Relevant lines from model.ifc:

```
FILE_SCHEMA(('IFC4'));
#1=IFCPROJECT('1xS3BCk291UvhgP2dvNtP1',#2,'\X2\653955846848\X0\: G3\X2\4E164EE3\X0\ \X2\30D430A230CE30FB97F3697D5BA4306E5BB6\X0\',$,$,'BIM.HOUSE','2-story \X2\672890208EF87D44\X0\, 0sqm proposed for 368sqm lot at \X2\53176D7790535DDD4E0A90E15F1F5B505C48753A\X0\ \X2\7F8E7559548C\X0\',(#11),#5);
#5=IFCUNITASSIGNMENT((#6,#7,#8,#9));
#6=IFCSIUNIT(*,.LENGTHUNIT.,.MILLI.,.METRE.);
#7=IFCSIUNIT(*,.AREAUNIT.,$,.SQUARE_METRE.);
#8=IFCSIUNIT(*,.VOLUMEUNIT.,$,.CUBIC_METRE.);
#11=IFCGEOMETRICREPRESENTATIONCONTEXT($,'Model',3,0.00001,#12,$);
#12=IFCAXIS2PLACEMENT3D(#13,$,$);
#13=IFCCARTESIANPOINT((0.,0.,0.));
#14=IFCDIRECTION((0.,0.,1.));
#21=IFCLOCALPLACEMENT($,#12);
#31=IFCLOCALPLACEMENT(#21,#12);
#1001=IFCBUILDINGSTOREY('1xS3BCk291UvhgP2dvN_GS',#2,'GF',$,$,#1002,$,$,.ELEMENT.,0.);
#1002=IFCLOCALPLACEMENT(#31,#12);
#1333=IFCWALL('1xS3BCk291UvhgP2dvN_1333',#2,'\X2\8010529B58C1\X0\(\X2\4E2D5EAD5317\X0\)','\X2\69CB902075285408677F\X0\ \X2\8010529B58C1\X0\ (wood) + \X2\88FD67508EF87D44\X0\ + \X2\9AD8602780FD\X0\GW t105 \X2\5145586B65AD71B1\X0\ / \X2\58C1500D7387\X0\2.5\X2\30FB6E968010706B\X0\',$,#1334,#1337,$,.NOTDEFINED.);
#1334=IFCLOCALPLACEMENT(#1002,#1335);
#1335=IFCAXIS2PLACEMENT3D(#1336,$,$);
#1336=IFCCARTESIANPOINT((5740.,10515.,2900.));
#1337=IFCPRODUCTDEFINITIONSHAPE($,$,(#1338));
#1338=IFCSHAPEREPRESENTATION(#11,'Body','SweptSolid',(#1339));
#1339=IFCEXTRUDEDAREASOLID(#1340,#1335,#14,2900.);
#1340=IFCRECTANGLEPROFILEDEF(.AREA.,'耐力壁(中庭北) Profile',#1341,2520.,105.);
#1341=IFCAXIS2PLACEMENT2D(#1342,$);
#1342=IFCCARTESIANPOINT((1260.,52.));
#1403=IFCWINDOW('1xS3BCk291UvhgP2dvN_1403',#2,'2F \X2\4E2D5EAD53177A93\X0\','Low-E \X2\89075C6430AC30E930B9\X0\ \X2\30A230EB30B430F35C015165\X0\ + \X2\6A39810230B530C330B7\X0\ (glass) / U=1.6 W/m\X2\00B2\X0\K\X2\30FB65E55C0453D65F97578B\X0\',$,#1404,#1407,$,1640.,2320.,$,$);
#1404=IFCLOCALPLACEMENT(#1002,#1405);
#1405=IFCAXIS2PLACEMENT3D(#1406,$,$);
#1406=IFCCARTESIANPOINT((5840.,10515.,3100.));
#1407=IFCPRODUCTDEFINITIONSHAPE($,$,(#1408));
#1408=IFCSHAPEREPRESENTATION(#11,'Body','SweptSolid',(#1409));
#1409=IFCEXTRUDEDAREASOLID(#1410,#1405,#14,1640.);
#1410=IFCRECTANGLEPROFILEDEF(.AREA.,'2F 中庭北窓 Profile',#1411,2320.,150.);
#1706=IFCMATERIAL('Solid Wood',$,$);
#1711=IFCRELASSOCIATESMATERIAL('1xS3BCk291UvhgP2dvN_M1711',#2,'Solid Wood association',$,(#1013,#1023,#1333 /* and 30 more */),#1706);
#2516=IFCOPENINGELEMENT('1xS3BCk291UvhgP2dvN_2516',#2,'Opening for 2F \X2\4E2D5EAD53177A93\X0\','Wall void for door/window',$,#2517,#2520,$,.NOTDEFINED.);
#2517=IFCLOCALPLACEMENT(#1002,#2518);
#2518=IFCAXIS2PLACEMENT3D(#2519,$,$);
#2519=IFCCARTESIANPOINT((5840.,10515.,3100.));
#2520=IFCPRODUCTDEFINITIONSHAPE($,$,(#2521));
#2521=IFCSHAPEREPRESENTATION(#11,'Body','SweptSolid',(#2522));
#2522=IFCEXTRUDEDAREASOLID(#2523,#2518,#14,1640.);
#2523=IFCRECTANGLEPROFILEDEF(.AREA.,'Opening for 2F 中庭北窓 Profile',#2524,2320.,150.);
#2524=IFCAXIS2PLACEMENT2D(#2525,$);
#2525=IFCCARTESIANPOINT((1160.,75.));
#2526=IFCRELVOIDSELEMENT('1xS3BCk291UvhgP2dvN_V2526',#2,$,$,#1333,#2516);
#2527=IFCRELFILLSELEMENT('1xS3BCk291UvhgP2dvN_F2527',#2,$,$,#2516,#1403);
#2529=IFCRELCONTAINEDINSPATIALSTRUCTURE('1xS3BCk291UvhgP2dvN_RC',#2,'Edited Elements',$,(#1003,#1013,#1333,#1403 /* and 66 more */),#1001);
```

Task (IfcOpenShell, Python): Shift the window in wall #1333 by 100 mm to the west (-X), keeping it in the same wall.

```python
import ifcopenshell
import ifcopenshell.api.geometry
import ifcopenshell.util.placement
import ifcopenshell.util.unit

model = ifcopenshell.open("model.ifc")
unit_scale = ifcopenshell.util.unit.calculate_unit_scale(model)

window = model.by_id(1403)
opening = window.FillsVoids[0].RelatingOpeningElement
wall = opening.VoidsElements[0].RelatingBuildingElement

wall_matrix = ifcopenshell.util.placement.get_local_placement(wall.ObjectPlacement)
shift = wall_matrix[:3, 0] * -0.1 / unit_scale
before = ifcopenshell.util.placement.get_local_placement(window.ObjectPlacement)[:3, 3].copy()

# The window is not placed relative to its opening, so move both.
for product in (opening, window):
    matrix = ifcopenshell.util.placement.get_local_placement(product.ObjectPlacement)
    matrix[:3, 3] += shift
    ifcopenshell.api.geometry.edit_object_placement(model, product=product, matrix=matrix, is_si=False)

after = ifcopenshell.util.placement.get_local_placement(window.ObjectPlacement)[:3, 3]
print("window moved by", (after - before).round(3) + 0.0)

model.write("model_edited.ifc")
```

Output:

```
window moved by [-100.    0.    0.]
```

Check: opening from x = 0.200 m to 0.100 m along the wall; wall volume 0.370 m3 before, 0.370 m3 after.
